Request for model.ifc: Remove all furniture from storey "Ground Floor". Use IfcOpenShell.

First a look at what the model holds.

```python
import ifcopenshell
import ifcopenshell.util.element

model = ifcopenshell.open("model.ifc")
print(model.schema)
storey = next(s for s in model.by_type("IfcBuildingStorey") if s.Name == "Ground Floor")
furniture = [e for e in ifcopenshell.util.element.get_decomposition(storey) if e.is_a("IfcFurnishingElement")]
seen = {}
for e in furniture:
    element_type = ifcopenshell.util.element.get_type(e)
    name = element_type.Name if element_type not in (None, e) else None
    seen[name] = seen.get(name, 0) + 1
for name, count in sorted(seen.items(), key=str):
    print(count, "x", name)
```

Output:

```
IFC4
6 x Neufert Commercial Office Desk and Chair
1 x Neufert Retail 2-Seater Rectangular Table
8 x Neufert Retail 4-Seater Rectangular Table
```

```python
import ifcopenshell
import ifcopenshell.api.root
import ifcopenshell.util.element

model = ifcopenshell.open("model.ifc")

storey = next(s for s in model.by_type("IfcBuildingStorey") if s.Name == "Ground Floor")
furniture = [e for e in ifcopenshell.util.element.get_decomposition(storey) if e.is_a("IfcFurnishingElement")]

for e in furniture:
    ifcopenshell.api.root.remove_product(model, product=e)
print(len(furniture), "removed")

model.write("model_edited.ifc")
```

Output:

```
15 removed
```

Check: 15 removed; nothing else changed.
